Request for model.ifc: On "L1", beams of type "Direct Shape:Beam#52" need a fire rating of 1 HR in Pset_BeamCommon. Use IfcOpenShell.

First a look at what the model holds.

```python
import ifcopenshell
import ifcopenshell.util.element

model = ifcopenshell.open("model.ifc")
print(model.schema)
storey = next(s for s in model.by_type("IfcBuildingStorey") if s.Name == "L1")
beams = [e for e in ifcopenshell.util.element.get_decomposition(storey) if e.is_a("IfcBeam")]
seen = {}
for e in beams:
    element_type = ifcopenshell.util.element.get_type(e)
    key = (element_type.Name if element_type != e and element_type else None, ifcopenshell.util.element.get_pset(e, "Pset_BeamCommon", "FireRating"))
    seen[key] = seen.get(key, 0) + 1
for (name, value), count in sorted(seen.items(), key=str):
    print(count, "x", name, "|", value)
```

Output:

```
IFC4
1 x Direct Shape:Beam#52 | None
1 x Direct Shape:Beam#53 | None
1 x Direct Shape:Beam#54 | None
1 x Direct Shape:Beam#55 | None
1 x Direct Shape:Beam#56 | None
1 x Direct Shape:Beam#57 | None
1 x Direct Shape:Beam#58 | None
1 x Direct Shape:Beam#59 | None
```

```python
import ifcopenshell
import ifcopenshell.api.pset
import ifcopenshell.util.element

model = ifcopenshell.open("model.ifc")

storey = next(s for s in model.by_type("IfcBuildingStorey") if s.Name == "L1")
beams = [e for e in ifcopenshell.util.element.get_decomposition(storey) if e.is_a("IfcBeam")]

count = 0
for e in beams:
    element_type = ifcopenshell.util.element.get_type(e)
    if element_type in (None, e) or element_type.Name != "Direct Shape:Beam#52":
        continue
    # add_pset returns the element's existing set when there is one.
    pset = ifcopenshell.api.pset.add_pset(model, product=e, name="Pset_BeamCommon")
    ifcopenshell.api.pset.edit_pset(model, pset=pset, properties={"FireRating": "1 HR"})
    count += 1

print(count, "beams updated")

model.write("model_edited.ifc")
```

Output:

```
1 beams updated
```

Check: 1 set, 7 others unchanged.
